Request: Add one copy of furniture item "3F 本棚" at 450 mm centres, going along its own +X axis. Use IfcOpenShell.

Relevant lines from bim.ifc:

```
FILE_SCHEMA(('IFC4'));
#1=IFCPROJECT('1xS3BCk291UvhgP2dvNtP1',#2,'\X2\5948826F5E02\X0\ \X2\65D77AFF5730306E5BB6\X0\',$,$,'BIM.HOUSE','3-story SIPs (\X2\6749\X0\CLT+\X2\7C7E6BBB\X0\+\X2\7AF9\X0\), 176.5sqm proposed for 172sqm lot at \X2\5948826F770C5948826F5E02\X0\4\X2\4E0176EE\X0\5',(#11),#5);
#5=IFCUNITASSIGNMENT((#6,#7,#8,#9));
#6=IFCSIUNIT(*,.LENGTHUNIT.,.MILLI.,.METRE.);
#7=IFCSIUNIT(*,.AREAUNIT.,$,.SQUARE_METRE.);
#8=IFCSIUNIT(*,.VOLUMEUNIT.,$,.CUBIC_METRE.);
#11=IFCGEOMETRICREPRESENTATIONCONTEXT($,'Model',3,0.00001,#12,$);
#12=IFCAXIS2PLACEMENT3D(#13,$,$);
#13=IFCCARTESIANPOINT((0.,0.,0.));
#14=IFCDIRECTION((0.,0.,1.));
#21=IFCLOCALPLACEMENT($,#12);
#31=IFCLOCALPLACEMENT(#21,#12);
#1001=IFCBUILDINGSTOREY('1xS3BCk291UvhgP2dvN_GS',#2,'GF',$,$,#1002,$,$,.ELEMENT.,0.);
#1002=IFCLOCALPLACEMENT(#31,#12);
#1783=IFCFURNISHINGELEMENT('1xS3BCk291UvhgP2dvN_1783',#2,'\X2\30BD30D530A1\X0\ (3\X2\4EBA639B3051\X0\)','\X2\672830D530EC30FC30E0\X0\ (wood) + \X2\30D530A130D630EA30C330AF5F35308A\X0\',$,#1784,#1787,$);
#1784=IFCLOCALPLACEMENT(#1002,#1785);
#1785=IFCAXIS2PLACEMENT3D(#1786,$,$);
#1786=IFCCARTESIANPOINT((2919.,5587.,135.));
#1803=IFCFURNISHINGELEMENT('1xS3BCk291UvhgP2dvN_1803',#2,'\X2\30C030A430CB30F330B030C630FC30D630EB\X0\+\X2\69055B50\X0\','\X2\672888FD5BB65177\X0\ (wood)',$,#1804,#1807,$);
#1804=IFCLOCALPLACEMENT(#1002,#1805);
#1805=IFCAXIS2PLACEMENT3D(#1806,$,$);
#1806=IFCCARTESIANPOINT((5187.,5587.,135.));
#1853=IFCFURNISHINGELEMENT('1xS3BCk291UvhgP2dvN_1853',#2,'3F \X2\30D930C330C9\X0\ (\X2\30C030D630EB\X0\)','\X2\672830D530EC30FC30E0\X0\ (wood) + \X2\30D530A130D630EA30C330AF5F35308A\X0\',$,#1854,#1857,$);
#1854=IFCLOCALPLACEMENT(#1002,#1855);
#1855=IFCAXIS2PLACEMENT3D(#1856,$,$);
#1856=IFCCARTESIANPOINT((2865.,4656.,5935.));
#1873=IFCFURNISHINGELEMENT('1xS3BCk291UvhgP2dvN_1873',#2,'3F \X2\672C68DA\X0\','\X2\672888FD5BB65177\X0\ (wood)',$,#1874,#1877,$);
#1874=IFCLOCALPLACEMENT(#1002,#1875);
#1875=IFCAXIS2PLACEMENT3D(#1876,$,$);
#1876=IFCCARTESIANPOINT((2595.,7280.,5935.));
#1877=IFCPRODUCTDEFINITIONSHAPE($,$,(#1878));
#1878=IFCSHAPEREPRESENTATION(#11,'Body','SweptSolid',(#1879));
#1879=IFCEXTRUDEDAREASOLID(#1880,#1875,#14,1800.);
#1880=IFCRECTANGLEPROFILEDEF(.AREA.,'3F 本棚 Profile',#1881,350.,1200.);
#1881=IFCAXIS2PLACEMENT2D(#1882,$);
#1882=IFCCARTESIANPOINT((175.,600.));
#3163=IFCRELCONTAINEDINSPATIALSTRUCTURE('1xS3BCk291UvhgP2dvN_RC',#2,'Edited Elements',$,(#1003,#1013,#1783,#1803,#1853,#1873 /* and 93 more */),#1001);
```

```python
import ifcopenshell
import ifcopenshell.api.geometry
import ifcopenshell.api.root
import ifcopenshell.util.element
import ifcopenshell.util.placement

model = ifcopenshell.open("bim.ifc")


def reuse_history(source, copy):
    """copy_class also copies each property set's owner history, people and application; keep the originals."""
    for rel in copy.IsDefinedBy:
        if rel.is_a("IfcRelDefinesByProperties") and (history := rel.RelatingPropertyDefinition.OwnerHistory):
            rel.RelatingPropertyDefinition.OwnerHistory = source.OwnerHistory
            ifcopenshell.util.element.remove_deep2(model, history)


source = model.by_guid("1xS3BCk291UvhgP2dvN_1873")
base = ifcopenshell.util.placement.get_local_placement(source.ObjectPlacement)
step = base[:3, 0] * 450.0

for i in range(1, 2):
    copy = ifcopenshell.api.root.copy_class(model, product=source)
    copy.Representation = ifcopenshell.util.element.copy_deep(
        model, source.Representation, exclude=["IfcGeometricRepresentationContext", "IfcRepresentationMap"]
    )
    reuse_history(source, copy)
    matrix = base.copy()
    matrix[:3, 3] += i * step
    print("added at", matrix[:3, 3].round(3) + 0.0)
    ifcopenshell.api.geometry.edit_object_placement(model, product=copy, matrix=matrix, is_si=False)

model.write("bim_v2.ifc")
```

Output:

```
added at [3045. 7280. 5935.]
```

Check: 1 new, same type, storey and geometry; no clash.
